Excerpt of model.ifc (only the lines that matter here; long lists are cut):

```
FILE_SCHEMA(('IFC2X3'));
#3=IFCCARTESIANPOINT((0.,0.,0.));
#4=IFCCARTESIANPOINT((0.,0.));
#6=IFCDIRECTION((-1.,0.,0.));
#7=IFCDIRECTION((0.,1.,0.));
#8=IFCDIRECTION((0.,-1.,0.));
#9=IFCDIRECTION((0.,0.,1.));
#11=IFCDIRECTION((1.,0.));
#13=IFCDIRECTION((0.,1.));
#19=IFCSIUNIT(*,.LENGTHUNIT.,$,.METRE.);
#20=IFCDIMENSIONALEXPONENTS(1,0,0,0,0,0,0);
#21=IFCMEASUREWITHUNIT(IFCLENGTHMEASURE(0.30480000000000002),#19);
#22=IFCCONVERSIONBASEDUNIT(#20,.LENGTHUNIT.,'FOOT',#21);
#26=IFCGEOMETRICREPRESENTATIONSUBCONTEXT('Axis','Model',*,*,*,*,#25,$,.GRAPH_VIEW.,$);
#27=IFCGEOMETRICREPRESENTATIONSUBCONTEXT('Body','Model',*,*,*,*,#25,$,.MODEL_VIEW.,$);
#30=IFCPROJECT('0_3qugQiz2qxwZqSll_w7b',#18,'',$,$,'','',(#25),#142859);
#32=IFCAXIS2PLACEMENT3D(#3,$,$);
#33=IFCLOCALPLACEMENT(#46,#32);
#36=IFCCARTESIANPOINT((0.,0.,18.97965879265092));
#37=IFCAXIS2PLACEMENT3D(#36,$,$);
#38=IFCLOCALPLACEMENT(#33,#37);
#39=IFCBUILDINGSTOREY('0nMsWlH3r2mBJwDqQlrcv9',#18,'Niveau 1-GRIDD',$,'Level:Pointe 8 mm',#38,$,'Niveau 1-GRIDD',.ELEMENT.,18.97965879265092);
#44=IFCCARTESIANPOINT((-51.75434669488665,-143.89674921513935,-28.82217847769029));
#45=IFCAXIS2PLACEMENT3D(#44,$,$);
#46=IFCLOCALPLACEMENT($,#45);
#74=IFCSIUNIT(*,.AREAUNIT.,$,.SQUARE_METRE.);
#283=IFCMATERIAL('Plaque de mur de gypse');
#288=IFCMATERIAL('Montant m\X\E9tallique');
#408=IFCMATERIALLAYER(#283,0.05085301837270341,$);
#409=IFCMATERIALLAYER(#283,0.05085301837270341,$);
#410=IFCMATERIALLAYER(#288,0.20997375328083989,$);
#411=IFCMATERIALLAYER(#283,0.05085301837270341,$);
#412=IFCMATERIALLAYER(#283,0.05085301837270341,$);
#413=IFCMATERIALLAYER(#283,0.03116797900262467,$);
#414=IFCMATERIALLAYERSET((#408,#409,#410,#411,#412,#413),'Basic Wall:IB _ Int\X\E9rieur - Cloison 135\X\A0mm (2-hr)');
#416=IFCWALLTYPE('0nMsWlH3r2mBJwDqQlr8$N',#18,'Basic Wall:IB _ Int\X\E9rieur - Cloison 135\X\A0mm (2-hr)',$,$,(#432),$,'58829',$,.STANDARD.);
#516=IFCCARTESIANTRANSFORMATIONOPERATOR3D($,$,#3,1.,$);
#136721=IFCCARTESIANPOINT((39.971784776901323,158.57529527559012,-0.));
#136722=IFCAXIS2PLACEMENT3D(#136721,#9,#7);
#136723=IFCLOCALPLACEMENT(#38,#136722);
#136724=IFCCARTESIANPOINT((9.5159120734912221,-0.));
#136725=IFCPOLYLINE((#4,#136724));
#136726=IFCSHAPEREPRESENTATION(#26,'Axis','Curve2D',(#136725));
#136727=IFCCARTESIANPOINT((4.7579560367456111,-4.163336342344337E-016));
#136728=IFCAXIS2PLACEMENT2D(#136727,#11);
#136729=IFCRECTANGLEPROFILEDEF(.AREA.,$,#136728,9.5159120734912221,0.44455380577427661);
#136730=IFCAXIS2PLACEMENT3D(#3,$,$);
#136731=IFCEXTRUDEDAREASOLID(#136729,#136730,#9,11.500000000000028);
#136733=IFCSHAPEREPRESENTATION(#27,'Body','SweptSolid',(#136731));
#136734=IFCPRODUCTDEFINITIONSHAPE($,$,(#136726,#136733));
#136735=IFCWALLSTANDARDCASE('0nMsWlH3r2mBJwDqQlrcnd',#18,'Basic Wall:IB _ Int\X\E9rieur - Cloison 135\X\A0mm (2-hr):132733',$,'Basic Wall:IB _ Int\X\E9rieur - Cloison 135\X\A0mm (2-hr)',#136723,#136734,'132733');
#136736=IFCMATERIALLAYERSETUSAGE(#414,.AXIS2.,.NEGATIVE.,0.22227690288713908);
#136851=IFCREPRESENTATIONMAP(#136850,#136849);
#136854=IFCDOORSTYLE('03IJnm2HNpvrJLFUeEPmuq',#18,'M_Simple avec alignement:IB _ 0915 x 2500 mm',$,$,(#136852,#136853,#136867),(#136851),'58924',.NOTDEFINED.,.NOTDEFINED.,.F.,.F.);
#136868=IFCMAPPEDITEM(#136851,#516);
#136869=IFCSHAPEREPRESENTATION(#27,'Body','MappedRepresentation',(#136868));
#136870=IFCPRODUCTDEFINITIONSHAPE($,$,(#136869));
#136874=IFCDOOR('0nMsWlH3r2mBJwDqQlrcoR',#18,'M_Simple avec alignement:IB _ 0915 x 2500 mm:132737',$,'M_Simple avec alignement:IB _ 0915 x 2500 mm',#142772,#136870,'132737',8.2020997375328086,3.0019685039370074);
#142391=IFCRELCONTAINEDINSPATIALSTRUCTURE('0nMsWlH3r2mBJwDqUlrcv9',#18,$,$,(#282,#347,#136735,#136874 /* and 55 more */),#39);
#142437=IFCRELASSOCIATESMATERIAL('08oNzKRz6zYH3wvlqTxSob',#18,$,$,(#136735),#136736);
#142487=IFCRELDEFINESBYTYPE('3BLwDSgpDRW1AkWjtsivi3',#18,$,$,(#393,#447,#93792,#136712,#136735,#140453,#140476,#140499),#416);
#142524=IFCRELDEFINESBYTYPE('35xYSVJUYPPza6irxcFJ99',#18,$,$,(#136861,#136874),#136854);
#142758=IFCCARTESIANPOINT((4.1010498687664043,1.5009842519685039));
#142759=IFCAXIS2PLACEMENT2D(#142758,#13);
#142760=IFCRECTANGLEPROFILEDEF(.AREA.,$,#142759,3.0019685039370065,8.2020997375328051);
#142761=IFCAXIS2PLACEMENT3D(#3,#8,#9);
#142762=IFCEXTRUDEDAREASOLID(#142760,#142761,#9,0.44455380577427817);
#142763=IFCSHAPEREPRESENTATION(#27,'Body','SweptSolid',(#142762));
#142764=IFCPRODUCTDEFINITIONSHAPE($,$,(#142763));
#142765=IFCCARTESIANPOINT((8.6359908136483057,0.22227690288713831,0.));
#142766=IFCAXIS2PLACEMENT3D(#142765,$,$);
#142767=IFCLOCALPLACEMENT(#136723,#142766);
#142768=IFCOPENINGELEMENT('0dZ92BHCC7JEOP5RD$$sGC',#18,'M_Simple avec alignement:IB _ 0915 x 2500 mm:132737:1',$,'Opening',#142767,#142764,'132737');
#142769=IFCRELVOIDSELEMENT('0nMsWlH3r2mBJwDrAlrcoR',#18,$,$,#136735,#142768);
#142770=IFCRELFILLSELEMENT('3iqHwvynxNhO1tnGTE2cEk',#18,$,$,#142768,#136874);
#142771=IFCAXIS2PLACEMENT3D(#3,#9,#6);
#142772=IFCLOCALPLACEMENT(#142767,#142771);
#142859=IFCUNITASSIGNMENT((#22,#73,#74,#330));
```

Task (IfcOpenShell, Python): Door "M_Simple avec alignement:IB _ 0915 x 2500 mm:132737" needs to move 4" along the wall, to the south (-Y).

```python
import ifcopenshell
import ifcopenshell.api.geometry
import ifcopenshell.util.placement
import ifcopenshell.util.unit

model = ifcopenshell.open("model.ifc")
unit_scale = ifcopenshell.util.unit.calculate_unit_scale(model)

door = model.by_id(136874)
opening = door.FillsVoids[0].RelatingOpeningElement
wall = opening.VoidsElements[0].RelatingBuildingElement

wall_matrix = ifcopenshell.util.placement.get_local_placement(wall.ObjectPlacement)
shift = wall_matrix[:3, 0] * -4 * 0.0254 / unit_scale
before = ifcopenshell.util.placement.get_local_placement(door.ObjectPlacement)[:3, 3].copy()

# The door is placed relative to its opening, so it follows when the opening moves.
matrix = ifcopenshell.util.placement.get_local_placement(opening.ObjectPlacement)
matrix[:3, 3] += shift
ifcopenshell.api.geometry.edit_object_placement(
    model, product=opening, matrix=matrix, is_si=False, should_transform_children=True
)

after = ifcopenshell.util.placement.get_local_placement(door.ObjectPlacement)[:3, 3]
print("door moved by", (after - before).round(3) + 0.0)

model.write("model-out.ifc")
```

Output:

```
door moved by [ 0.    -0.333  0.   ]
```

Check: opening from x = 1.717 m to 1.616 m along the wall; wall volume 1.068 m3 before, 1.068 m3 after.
